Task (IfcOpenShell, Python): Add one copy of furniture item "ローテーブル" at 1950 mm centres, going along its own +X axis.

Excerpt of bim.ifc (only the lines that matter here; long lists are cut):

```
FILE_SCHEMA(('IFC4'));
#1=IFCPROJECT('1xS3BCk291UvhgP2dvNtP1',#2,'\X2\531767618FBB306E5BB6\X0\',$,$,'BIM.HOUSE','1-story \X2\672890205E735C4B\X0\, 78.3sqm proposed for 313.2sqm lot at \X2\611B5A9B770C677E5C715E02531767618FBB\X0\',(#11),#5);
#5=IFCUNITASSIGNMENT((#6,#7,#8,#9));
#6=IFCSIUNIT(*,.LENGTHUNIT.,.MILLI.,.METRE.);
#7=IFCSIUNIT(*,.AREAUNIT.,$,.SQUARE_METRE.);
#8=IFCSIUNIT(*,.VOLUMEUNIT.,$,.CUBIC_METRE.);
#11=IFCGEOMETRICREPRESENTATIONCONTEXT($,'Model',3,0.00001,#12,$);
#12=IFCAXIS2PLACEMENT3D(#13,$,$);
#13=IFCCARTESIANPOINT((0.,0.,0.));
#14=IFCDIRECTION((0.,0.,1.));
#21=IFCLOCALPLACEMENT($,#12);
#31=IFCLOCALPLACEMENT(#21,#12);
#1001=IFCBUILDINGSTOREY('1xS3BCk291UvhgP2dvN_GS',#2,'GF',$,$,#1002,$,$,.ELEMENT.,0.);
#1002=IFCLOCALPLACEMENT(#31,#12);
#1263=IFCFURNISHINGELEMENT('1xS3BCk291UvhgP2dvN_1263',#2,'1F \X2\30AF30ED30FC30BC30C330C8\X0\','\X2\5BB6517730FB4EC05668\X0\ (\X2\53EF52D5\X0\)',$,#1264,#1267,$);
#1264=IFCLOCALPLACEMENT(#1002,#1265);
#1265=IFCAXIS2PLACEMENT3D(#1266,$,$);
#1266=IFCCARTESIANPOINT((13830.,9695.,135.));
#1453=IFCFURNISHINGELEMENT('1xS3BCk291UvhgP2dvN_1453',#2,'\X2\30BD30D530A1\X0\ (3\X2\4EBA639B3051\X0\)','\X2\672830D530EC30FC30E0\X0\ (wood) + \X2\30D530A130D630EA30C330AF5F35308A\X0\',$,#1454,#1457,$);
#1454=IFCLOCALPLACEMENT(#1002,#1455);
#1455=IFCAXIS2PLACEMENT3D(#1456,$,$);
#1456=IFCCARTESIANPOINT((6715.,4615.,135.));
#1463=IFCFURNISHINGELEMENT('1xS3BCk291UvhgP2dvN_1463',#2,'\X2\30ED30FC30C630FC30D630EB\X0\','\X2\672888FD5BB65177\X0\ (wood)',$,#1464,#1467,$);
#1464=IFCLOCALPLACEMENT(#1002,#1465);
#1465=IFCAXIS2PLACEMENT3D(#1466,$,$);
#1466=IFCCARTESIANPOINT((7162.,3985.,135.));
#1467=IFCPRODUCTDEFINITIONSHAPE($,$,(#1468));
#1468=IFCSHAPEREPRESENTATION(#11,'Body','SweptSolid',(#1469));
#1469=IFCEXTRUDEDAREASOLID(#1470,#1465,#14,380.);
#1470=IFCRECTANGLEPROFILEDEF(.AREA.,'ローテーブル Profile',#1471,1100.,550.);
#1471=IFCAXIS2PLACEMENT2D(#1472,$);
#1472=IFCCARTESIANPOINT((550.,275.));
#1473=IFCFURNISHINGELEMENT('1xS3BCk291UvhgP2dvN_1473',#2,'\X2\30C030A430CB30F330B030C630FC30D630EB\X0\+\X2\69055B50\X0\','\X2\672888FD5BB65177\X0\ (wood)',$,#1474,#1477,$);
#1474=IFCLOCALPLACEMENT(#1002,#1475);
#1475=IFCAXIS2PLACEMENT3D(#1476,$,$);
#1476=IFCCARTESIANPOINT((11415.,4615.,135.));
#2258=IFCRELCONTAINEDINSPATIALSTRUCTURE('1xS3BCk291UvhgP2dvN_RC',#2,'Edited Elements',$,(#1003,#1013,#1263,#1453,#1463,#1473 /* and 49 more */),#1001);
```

```python
import ifcopenshell
import ifcopenshell.api.geometry
import ifcopenshell.api.root
import ifcopenshell.util.element
import ifcopenshell.util.placement
import ifcopenshell.util.unit

model = ifcopenshell.open("bim.ifc")
unit_scale = ifcopenshell.util.unit.calculate_unit_scale(model)


def reuse_history(source, copy):
    """copy_class also copies each property set's owner history, people and application; keep the originals."""
    for rel in copy.IsDefinedBy:
        if rel.is_a("IfcRelDefinesByProperties") and (history := rel.RelatingPropertyDefinition.OwnerHistory):
            rel.RelatingPropertyDefinition.OwnerHistory = source.OwnerHistory
            ifcopenshell.util.element.remove_deep2(model, history)


source = model.by_guid("1xS3BCk291UvhgP2dvN_1463")
base = ifcopenshell.util.placement.get_local_placement(source.ObjectPlacement)
step = base[:3, 0] * 1.95 / unit_scale

for i in range(1, 2):
    copy = ifcopenshell.api.root.copy_class(model, product=source)
    copy.Representation = ifcopenshell.util.element.copy_deep(
        model, source.Representation, exclude=["IfcGeometricRepresentationContext", "IfcRepresentationMap"]
    )
    reuse_history(source, copy)
    matrix = base.copy()
    matrix[:3, 3] += i * step
    print("added at", matrix[:3, 3].round(3) + 0.0)
    ifcopenshell.api.geometry.edit_object_placement(model, product=copy, matrix=matrix, is_si=False)

model.write("bim_v2.ifc")
```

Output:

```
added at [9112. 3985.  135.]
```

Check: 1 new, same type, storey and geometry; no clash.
